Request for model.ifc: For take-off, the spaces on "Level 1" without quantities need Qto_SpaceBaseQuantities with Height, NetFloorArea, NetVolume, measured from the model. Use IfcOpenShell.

First a look at what the model holds.

```python
import ifcopenshell
import ifcopenshell.util.element
import ifcopenshell.util.unit

model = ifcopenshell.open("model.ifc")
print(model.schema)
for unit_type in ("LENGTHUNIT", "AREAUNIT", "VOLUMEUNIT"):
    print(unit_type, ifcopenshell.util.unit.calculate_unit_scale(model, unit_type))
storey = next(s for s in model.by_type("IfcBuildingStorey") if s.Name == "Level 1")
spaces = [e for e in ifcopenshell.util.element.get_decomposition(storey) if e.is_a("IfcSpace")]
for e in sorted(spaces, key=lambda e: e.id()):
    print(e.id(), e.is_a(), e.Name, list(ifcopenshell.util.element.get_psets(e, qtos_only=True)), sep=" | ")
```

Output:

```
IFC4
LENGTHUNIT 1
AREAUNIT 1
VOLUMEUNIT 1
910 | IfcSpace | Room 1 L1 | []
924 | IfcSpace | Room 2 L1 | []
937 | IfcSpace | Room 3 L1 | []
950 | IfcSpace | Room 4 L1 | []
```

```python
import ifcopenshell
import ifcopenshell.api.pset
import ifcopenshell.geom
import ifcopenshell.util.element
import ifcopenshell.util.shape
import ifcopenshell.util.unit

model = ifcopenshell.open("model.ifc")
unit_scale = ifcopenshell.util.unit.calculate_unit_scale(model)
area_scale = ifcopenshell.util.unit.calculate_unit_scale(model, "AREAUNIT")
volume_scale = ifcopenshell.util.unit.calculate_unit_scale(model, "VOLUMEUNIT")
settings = ifcopenshell.geom.settings()

storey = next(s for s in model.by_type("IfcBuildingStorey") if s.Name == "Level 1")
spaces = [e for e in ifcopenshell.util.element.get_decomposition(storey) if e.is_a("IfcSpace")]

for e in sorted(spaces, key=lambda e: e.id()):
    if ifcopenshell.util.element.get_psets(e, qtos_only=True, should_inherit=False):
        continue
    # Geometry comes back in metres, in the element's own axes.
    shape = ifcopenshell.geom.create_shape(settings, e)
    values = {
        "Height": ifcopenshell.util.shape.get_z(shape.geometry) / unit_scale,
        "NetFloorArea": ifcopenshell.util.shape.get_footprint_area(shape.geometry) / area_scale,
        "NetVolume": ifcopenshell.util.shape.get_volume(shape.geometry) / volume_scale,
    }
    qto = ifcopenshell.api.pset.add_qto(model, product=e, name="Qto_SpaceBaseQuantities")
    ifcopenshell.api.pset.edit_qto(model, qto=qto, properties=values)
    print(e.id(), {k: round(v, 3) for k, v in values.items()})

model.write("model_edited.ifc")
```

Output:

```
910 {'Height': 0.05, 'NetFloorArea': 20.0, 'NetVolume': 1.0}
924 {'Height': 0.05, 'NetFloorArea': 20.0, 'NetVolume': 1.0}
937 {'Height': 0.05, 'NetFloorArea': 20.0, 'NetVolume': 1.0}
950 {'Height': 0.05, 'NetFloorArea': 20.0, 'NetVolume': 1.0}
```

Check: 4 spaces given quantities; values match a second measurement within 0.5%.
